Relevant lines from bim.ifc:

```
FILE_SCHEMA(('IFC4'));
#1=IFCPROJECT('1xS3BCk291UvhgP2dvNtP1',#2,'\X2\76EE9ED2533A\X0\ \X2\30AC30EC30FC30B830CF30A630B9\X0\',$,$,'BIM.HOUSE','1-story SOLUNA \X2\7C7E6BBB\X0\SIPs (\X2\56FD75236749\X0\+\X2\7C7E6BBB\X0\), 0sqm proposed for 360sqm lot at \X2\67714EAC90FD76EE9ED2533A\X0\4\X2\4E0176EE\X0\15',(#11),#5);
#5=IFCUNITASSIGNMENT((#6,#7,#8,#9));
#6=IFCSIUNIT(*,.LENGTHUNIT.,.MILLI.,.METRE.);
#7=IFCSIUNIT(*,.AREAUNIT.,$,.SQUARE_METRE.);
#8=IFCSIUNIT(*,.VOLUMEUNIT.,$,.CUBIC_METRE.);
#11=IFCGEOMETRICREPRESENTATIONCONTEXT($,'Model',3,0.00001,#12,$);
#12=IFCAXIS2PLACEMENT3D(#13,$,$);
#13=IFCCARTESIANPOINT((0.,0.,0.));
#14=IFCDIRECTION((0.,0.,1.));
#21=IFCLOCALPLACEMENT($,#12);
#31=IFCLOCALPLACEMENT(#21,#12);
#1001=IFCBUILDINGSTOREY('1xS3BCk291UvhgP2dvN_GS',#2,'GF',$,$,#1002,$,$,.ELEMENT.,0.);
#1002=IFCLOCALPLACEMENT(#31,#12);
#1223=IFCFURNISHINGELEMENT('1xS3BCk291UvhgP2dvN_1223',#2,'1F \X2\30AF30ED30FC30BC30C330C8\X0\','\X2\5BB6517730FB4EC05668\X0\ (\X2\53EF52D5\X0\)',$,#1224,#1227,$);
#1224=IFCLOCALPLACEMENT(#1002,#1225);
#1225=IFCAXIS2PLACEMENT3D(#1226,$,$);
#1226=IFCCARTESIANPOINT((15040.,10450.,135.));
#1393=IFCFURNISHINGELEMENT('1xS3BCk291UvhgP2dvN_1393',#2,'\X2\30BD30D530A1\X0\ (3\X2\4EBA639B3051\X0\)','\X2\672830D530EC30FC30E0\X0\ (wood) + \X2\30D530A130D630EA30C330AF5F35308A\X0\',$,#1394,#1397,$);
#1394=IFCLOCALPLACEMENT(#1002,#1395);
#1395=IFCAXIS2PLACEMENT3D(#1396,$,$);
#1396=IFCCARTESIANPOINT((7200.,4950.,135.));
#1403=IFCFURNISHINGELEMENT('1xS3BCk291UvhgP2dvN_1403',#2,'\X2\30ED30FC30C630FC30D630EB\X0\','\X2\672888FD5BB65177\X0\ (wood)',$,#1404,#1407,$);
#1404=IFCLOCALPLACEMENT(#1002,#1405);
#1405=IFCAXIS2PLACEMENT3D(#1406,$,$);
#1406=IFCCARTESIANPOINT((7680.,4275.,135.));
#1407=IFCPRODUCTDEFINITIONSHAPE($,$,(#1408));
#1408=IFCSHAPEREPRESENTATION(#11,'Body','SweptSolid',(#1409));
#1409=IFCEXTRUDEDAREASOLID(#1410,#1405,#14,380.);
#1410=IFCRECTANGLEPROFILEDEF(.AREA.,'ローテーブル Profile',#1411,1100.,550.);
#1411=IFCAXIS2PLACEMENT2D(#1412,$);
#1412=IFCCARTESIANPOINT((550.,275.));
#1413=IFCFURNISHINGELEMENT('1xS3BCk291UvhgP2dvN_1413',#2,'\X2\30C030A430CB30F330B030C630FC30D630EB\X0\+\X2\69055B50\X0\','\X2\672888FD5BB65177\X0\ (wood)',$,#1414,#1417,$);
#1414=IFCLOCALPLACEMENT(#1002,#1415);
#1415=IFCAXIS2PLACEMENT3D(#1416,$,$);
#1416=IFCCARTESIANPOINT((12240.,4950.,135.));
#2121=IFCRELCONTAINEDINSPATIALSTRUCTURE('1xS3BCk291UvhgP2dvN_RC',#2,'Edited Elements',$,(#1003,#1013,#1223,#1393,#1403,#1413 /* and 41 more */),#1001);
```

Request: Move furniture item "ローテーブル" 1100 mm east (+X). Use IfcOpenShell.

```python
import ifcopenshell
import ifcopenshell.api.geometry
import ifcopenshell.util.placement

model = ifcopenshell.open("bim.ifc")

item = model.by_guid("1xS3BCk291UvhgP2dvN_1403")
matrix = ifcopenshell.util.placement.get_local_placement(item.ObjectPlacement)
matrix[0, 3] += 1100.0
ifcopenshell.api.geometry.edit_object_placement(model, product=item, matrix=matrix, is_si=False)

print(ifcopenshell.util.placement.get_local_placement(item.ObjectPlacement).round(3) + 0.0)

model.write("bim_rev.ifc")
```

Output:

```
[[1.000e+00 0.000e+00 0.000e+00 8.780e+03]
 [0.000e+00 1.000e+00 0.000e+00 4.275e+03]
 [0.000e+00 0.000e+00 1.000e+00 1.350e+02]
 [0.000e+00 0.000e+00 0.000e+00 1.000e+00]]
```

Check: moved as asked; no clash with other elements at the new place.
